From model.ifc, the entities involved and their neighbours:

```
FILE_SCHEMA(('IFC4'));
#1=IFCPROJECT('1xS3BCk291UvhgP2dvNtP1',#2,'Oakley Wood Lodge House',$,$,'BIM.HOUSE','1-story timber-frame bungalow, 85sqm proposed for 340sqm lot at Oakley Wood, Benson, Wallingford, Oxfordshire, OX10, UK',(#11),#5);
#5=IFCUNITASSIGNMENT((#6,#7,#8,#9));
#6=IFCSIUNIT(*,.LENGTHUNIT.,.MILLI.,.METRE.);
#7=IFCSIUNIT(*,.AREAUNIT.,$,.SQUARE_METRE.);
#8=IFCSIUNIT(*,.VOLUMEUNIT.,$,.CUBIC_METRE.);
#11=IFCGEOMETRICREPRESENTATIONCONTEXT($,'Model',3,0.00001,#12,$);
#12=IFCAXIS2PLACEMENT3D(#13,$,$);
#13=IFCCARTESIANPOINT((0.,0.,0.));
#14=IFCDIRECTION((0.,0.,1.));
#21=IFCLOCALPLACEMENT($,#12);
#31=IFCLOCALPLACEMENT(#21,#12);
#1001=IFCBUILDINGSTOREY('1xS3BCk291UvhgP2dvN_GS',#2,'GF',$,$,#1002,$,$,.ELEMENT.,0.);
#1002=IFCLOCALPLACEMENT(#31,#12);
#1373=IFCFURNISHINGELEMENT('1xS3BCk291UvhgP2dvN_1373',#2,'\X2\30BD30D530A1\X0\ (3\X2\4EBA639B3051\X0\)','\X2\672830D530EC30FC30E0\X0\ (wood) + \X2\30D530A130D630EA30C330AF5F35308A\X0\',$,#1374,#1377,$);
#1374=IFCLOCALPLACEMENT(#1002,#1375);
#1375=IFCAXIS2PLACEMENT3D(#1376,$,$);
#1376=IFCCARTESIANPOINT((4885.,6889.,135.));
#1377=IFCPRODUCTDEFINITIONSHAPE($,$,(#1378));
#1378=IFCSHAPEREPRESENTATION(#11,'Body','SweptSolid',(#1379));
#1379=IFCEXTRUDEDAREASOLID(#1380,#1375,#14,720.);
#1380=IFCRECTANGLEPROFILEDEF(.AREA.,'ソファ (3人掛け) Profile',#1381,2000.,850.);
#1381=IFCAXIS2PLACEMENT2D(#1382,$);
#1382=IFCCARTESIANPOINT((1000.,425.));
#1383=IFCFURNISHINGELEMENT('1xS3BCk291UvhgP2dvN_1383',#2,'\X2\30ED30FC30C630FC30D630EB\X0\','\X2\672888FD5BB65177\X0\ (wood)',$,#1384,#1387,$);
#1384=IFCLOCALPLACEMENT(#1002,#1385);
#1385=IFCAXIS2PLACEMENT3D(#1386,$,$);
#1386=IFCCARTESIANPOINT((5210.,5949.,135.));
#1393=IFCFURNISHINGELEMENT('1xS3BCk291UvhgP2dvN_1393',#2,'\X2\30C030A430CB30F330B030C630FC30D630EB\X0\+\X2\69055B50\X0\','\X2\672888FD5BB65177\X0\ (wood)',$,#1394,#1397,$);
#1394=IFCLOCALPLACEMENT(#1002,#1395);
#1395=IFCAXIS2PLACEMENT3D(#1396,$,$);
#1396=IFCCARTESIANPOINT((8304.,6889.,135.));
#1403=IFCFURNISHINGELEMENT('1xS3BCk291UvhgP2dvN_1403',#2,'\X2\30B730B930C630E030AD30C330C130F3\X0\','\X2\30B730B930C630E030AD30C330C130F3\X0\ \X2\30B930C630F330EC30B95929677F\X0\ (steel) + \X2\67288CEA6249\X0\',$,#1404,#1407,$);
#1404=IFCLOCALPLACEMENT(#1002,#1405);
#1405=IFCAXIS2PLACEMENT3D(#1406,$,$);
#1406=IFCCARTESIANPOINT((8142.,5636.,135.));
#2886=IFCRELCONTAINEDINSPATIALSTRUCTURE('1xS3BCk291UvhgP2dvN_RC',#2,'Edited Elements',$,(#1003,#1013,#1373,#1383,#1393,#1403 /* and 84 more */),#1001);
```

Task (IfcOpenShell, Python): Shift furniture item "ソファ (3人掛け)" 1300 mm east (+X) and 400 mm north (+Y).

```python
import ifcopenshell
import ifcopenshell.api.geometry
import ifcopenshell.util.placement

model = ifcopenshell.open("model.ifc")

item = model.by_guid("1xS3BCk291UvhgP2dvN_1373")
matrix = ifcopenshell.util.placement.get_local_placement(item.ObjectPlacement)
matrix[0, 3] += 1300.0
matrix[1, 3] += 400.0
ifcopenshell.api.geometry.edit_object_placement(model, product=item, matrix=matrix, is_si=False)

print(ifcopenshell.util.placement.get_local_placement(item.ObjectPlacement).round(3) + 0.0)

model.write("model_rev.ifc")
```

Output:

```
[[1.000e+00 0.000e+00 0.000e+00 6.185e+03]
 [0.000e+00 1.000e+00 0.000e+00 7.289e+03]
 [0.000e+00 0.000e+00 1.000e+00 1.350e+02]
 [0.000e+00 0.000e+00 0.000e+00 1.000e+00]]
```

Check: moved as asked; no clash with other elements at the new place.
